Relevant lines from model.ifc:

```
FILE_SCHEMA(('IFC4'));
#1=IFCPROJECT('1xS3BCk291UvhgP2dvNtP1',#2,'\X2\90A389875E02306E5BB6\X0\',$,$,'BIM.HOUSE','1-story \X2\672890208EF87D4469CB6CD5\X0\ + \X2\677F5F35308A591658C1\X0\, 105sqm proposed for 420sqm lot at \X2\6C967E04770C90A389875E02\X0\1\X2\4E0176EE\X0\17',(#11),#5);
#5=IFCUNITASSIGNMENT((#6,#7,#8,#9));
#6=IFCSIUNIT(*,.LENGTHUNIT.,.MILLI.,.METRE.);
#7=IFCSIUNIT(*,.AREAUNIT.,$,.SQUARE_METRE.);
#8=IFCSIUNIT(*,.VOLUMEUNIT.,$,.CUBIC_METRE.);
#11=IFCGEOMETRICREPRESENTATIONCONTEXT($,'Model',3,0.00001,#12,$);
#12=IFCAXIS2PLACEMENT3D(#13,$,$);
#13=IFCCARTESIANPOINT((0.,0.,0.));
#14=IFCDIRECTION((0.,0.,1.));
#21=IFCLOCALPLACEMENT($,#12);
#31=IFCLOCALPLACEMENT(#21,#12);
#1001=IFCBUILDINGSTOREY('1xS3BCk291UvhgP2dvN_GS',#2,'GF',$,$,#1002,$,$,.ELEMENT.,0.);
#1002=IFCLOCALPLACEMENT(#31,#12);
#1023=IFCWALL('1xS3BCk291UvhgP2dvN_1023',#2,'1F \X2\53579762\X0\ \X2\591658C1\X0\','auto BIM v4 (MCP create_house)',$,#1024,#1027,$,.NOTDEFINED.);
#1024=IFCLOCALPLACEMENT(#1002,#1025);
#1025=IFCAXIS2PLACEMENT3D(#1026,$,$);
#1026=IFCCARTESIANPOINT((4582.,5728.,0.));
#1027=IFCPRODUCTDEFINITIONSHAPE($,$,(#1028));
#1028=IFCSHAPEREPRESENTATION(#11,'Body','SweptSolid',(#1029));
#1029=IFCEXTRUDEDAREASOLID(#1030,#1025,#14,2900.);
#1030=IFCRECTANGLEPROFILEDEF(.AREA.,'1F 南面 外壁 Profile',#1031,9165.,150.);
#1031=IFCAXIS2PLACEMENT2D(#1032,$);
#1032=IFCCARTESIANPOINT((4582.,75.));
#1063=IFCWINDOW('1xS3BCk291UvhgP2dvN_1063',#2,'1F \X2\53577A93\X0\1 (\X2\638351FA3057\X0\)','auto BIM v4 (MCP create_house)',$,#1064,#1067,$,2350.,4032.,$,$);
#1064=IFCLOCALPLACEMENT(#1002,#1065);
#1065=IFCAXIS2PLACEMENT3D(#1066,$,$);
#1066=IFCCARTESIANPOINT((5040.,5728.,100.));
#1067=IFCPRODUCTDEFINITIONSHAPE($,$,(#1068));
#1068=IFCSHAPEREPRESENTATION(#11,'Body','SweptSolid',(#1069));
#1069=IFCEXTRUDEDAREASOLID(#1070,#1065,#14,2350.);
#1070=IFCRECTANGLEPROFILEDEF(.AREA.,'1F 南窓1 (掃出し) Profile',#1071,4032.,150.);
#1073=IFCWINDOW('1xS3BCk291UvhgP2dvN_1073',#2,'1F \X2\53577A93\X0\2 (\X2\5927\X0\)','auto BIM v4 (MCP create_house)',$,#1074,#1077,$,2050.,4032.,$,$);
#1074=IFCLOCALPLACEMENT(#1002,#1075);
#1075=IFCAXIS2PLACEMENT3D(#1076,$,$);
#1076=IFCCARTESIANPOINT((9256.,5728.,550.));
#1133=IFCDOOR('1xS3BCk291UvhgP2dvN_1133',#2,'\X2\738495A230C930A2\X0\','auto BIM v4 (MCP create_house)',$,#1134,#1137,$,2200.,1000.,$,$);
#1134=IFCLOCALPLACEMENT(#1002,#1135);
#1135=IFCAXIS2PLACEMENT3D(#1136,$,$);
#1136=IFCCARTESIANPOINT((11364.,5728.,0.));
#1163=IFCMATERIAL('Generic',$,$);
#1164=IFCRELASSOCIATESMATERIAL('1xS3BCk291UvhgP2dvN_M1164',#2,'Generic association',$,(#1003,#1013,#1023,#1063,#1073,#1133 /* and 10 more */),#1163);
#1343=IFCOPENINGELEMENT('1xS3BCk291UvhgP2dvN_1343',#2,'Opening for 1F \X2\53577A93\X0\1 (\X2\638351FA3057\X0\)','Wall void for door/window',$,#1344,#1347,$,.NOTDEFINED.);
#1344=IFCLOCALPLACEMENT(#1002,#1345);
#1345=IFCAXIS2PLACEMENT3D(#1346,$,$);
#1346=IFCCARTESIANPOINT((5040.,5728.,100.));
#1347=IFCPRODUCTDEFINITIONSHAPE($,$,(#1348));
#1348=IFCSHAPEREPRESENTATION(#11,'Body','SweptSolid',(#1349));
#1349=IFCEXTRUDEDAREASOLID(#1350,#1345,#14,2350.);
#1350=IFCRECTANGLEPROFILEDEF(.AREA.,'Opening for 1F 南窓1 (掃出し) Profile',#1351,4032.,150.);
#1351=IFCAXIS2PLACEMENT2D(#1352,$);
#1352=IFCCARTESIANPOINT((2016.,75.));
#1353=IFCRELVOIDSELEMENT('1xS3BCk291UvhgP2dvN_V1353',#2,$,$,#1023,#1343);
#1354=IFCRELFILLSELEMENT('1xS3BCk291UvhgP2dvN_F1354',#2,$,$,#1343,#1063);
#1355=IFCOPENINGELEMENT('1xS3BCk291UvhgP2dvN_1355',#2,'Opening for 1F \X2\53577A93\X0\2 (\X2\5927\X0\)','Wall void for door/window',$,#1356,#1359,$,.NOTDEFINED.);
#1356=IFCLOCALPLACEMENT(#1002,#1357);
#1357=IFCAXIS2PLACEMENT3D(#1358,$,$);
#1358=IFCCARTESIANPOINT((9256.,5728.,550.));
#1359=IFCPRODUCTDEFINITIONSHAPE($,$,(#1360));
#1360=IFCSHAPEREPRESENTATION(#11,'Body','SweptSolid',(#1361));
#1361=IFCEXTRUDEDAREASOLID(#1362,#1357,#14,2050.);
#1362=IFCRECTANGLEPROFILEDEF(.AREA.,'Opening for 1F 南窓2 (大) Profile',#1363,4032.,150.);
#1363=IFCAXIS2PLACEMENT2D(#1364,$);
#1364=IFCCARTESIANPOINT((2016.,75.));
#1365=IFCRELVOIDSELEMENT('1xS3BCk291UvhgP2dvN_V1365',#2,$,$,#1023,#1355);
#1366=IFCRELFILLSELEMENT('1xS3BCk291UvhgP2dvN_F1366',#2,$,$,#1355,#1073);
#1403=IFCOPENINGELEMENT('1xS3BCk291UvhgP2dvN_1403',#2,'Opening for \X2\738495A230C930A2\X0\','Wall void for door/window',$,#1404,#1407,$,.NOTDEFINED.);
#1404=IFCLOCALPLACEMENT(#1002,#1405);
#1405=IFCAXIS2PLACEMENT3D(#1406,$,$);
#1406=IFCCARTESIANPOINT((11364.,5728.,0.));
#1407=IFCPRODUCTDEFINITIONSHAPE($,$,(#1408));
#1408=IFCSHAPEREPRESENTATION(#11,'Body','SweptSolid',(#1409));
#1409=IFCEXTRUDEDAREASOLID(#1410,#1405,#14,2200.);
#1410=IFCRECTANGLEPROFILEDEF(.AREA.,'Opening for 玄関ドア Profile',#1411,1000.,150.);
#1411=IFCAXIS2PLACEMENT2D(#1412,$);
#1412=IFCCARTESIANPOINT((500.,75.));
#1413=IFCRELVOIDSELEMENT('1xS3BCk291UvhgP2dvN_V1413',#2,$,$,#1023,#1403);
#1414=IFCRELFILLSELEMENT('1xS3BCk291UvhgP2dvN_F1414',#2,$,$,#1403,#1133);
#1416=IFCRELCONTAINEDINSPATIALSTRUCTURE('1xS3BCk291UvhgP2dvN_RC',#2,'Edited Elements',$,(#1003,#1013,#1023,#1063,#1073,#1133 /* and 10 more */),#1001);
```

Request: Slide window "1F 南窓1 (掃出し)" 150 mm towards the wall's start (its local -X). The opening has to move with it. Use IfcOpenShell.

```python
import ifcopenshell
import ifcopenshell.api.geometry
import ifcopenshell.util.placement
import ifcopenshell.util.unit

model = ifcopenshell.open("model.ifc")
unit_scale = ifcopenshell.util.unit.calculate_unit_scale(model)

window = model.by_guid("1xS3BCk291UvhgP2dvN_1063")
opening = window.FillsVoids[0].RelatingOpeningElement
wall = opening.VoidsElements[0].RelatingBuildingElement

wall_matrix = ifcopenshell.util.placement.get_local_placement(wall.ObjectPlacement)
shift = wall_matrix[:3, 0] * -0.15 / unit_scale
before = ifcopenshell.util.placement.get_local_placement(window.ObjectPlacement)[:3, 3].copy()

# The window is not placed relative to its opening, so move both.
for product in (opening, window):
    matrix = ifcopenshell.util.placement.get_local_placement(product.ObjectPlacement)
    matrix[:3, 3] += shift
    ifcopenshell.api.geometry.edit_object_placement(model, product=product, matrix=matrix, is_si=False)

after = ifcopenshell.util.placement.get_local_placement(window.ObjectPlacement)[:3, 3]
print("window moved by", (after - before).round(3) + 0.0)

model.write("model-out.ifc")
```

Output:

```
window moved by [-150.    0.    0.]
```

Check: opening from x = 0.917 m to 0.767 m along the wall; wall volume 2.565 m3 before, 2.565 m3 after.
